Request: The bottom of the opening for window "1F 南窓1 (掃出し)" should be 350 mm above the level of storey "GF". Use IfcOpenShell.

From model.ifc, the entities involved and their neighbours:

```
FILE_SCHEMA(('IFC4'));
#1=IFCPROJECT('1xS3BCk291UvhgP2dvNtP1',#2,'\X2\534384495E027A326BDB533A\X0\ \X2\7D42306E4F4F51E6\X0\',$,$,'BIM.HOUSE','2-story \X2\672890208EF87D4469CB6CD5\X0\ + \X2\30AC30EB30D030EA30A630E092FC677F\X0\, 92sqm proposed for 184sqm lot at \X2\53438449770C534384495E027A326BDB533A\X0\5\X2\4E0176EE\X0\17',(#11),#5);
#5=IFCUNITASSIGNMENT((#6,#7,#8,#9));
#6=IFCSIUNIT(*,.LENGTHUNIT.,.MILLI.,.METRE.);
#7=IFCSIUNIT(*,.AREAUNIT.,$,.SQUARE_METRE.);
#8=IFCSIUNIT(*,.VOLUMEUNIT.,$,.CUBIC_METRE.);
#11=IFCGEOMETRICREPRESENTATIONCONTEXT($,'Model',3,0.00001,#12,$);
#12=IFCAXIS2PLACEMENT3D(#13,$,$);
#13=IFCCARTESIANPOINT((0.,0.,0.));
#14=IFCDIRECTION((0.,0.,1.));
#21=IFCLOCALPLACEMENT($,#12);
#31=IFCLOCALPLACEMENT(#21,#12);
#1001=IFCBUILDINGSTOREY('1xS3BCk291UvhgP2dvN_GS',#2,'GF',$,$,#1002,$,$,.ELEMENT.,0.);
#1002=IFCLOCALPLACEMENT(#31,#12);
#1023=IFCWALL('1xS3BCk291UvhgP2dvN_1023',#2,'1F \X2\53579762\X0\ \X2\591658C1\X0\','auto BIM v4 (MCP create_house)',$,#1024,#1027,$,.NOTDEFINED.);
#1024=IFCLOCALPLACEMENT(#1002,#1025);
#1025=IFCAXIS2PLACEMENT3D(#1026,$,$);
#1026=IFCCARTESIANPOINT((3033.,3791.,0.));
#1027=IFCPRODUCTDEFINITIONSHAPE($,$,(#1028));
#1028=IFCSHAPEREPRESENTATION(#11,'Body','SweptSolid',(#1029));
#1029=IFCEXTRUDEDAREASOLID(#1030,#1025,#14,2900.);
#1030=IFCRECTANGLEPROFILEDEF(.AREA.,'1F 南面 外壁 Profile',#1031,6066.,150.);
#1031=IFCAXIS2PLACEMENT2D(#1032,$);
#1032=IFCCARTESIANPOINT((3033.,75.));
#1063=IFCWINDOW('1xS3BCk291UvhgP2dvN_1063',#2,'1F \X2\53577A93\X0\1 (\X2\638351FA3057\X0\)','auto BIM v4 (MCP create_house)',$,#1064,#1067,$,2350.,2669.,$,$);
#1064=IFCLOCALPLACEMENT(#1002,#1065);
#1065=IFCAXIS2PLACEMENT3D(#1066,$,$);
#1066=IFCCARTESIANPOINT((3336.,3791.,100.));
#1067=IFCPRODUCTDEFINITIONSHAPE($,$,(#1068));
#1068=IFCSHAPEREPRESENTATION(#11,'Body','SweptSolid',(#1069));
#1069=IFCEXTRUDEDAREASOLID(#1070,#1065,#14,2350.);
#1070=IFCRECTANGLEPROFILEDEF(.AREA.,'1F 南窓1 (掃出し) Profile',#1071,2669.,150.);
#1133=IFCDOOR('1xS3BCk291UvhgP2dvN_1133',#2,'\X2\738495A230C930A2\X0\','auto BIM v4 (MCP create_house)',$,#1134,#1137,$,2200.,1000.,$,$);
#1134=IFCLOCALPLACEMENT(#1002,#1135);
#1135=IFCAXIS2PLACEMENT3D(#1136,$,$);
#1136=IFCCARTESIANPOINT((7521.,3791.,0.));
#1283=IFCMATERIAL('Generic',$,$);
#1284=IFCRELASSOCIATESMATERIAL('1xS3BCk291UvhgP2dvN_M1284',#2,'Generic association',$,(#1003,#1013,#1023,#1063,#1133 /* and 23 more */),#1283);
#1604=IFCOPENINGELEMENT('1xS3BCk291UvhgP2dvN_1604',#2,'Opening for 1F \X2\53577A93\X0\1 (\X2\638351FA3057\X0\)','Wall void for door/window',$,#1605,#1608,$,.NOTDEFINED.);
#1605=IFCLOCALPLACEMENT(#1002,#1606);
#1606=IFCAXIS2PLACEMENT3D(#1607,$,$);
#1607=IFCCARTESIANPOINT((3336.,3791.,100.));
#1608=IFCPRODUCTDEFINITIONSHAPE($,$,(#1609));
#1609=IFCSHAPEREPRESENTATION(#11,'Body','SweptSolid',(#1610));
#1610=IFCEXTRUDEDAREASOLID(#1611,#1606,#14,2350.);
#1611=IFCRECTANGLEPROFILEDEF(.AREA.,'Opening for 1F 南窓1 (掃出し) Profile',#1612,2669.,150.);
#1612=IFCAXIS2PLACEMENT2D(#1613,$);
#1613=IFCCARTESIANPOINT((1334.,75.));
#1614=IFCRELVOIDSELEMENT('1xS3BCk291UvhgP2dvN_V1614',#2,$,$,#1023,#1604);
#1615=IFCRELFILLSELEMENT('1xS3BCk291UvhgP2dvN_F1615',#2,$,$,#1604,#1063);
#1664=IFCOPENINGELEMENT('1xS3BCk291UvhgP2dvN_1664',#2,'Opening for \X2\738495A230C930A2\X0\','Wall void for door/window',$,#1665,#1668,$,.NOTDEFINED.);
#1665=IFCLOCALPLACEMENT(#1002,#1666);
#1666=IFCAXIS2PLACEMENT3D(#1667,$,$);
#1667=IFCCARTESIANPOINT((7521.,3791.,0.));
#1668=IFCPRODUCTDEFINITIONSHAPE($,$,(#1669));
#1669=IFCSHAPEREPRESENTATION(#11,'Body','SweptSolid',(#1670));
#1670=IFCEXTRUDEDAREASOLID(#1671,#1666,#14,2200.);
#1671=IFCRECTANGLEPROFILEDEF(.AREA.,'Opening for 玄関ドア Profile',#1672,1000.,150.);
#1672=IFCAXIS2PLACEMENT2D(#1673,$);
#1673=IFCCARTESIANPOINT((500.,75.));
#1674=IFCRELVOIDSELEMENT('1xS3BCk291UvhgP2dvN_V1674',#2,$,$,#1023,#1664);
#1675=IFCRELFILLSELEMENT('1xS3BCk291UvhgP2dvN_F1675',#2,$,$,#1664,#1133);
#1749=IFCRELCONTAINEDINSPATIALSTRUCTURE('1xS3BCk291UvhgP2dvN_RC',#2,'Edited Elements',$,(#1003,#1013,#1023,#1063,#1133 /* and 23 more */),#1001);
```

```python
import numpy as np
import ifcopenshell
import ifcopenshell.api.geometry
import ifcopenshell.geom
import ifcopenshell.util.element
import ifcopenshell.util.placement
import ifcopenshell.util.shape
import ifcopenshell.util.unit

model = ifcopenshell.open("model.ifc")
unit_scale = ifcopenshell.util.unit.calculate_unit_scale(model)

window = model.by_guid("1xS3BCk291UvhgP2dvN_1063")
opening = window.FillsVoids[0].RelatingOpeningElement
storey = ifcopenshell.util.element.get_container(window, ifc_class="IfcBuildingStorey")
level = ifcopenshell.util.placement.get_local_placement(storey.ObjectPlacement)[2, 3]

# The opening's origin need not be at the sill, so measure its lowest point.
shape = ifcopenshell.geom.create_shape(ifcopenshell.geom.settings(), opening)
bottom = ifcopenshell.util.shape.get_shape_bottom_elevation(shape, shape.geometry) / unit_scale
dz = level + 350.0 - bottom

shift = np.array([0.0, 0.0, dz])
# The window is not placed relative to its opening, so move both.
for product in (opening, window):
    matrix = ifcopenshell.util.placement.get_local_placement(product.ObjectPlacement)
    matrix[:3, 3] += shift
    ifcopenshell.api.geometry.edit_object_placement(model, product=product, matrix=matrix, is_si=False)

print(f"moved by {dz * unit_scale:+.3f} m")

model.write("model_updated.ifc")
```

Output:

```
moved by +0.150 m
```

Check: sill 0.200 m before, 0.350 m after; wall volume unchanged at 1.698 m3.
